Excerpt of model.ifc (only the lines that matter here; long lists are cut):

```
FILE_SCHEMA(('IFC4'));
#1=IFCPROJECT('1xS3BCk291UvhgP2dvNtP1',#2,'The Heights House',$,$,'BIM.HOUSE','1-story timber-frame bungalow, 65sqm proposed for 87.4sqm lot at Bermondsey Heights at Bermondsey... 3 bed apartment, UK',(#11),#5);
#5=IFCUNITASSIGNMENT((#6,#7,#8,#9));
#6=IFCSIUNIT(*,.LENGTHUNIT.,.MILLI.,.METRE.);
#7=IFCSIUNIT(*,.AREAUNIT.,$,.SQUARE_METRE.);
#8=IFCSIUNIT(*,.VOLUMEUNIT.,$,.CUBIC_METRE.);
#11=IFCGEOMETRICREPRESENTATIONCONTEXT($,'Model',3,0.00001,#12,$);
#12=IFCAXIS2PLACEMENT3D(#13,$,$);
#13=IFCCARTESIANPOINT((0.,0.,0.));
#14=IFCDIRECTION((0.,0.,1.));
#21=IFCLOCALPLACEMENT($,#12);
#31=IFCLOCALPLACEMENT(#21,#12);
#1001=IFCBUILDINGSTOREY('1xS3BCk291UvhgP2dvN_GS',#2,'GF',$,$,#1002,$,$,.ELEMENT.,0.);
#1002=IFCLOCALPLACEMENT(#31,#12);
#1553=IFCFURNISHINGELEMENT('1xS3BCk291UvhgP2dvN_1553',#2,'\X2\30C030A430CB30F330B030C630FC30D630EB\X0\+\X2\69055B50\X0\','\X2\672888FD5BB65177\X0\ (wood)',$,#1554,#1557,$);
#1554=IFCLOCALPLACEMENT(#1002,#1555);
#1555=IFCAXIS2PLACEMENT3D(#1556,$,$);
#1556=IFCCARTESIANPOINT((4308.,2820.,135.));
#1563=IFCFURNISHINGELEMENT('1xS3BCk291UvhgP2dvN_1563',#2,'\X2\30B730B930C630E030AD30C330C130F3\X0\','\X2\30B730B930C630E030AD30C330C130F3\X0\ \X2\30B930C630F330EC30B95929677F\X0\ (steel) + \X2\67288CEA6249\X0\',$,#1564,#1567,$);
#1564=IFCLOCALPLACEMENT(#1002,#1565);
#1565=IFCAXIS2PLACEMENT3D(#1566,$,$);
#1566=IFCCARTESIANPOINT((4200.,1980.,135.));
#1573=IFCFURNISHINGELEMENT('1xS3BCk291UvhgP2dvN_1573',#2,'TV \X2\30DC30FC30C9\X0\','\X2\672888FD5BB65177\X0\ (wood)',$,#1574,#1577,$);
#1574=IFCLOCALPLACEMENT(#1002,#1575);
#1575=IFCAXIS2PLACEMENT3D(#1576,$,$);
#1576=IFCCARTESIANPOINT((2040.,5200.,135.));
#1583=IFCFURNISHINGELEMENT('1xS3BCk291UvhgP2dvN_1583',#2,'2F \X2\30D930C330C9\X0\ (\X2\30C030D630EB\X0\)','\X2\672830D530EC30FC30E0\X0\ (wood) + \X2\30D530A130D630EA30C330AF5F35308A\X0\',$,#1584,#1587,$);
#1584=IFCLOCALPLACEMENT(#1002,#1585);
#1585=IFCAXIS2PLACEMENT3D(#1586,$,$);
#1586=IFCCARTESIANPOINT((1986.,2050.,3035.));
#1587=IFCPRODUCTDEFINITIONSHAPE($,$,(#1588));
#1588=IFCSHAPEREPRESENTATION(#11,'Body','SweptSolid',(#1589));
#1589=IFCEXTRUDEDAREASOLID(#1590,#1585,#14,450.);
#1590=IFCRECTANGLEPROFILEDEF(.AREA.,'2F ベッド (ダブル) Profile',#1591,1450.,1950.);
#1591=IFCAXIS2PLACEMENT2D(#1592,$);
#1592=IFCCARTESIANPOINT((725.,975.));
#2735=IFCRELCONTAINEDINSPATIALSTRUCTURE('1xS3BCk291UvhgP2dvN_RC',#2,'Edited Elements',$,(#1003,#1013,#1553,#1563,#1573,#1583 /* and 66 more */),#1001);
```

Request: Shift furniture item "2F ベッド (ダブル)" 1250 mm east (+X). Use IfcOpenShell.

```python
import ifcopenshell
import ifcopenshell.api.geometry
import ifcopenshell.util.placement

model = ifcopenshell.open("model.ifc")

item = model.by_id(1583)
matrix = ifcopenshell.util.placement.get_local_placement(item.ObjectPlacement)
matrix[0, 3] += 1250.0
ifcopenshell.api.geometry.edit_object_placement(model, product=item, matrix=matrix, is_si=False)

print(ifcopenshell.util.placement.get_local_placement(item.ObjectPlacement).round(3) + 0.0)

model.write("model-out.ifc")
```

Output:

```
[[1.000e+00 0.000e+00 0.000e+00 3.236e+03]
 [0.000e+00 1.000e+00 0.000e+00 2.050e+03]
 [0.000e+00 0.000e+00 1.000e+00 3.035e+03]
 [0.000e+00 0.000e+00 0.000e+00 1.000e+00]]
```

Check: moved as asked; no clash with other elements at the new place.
